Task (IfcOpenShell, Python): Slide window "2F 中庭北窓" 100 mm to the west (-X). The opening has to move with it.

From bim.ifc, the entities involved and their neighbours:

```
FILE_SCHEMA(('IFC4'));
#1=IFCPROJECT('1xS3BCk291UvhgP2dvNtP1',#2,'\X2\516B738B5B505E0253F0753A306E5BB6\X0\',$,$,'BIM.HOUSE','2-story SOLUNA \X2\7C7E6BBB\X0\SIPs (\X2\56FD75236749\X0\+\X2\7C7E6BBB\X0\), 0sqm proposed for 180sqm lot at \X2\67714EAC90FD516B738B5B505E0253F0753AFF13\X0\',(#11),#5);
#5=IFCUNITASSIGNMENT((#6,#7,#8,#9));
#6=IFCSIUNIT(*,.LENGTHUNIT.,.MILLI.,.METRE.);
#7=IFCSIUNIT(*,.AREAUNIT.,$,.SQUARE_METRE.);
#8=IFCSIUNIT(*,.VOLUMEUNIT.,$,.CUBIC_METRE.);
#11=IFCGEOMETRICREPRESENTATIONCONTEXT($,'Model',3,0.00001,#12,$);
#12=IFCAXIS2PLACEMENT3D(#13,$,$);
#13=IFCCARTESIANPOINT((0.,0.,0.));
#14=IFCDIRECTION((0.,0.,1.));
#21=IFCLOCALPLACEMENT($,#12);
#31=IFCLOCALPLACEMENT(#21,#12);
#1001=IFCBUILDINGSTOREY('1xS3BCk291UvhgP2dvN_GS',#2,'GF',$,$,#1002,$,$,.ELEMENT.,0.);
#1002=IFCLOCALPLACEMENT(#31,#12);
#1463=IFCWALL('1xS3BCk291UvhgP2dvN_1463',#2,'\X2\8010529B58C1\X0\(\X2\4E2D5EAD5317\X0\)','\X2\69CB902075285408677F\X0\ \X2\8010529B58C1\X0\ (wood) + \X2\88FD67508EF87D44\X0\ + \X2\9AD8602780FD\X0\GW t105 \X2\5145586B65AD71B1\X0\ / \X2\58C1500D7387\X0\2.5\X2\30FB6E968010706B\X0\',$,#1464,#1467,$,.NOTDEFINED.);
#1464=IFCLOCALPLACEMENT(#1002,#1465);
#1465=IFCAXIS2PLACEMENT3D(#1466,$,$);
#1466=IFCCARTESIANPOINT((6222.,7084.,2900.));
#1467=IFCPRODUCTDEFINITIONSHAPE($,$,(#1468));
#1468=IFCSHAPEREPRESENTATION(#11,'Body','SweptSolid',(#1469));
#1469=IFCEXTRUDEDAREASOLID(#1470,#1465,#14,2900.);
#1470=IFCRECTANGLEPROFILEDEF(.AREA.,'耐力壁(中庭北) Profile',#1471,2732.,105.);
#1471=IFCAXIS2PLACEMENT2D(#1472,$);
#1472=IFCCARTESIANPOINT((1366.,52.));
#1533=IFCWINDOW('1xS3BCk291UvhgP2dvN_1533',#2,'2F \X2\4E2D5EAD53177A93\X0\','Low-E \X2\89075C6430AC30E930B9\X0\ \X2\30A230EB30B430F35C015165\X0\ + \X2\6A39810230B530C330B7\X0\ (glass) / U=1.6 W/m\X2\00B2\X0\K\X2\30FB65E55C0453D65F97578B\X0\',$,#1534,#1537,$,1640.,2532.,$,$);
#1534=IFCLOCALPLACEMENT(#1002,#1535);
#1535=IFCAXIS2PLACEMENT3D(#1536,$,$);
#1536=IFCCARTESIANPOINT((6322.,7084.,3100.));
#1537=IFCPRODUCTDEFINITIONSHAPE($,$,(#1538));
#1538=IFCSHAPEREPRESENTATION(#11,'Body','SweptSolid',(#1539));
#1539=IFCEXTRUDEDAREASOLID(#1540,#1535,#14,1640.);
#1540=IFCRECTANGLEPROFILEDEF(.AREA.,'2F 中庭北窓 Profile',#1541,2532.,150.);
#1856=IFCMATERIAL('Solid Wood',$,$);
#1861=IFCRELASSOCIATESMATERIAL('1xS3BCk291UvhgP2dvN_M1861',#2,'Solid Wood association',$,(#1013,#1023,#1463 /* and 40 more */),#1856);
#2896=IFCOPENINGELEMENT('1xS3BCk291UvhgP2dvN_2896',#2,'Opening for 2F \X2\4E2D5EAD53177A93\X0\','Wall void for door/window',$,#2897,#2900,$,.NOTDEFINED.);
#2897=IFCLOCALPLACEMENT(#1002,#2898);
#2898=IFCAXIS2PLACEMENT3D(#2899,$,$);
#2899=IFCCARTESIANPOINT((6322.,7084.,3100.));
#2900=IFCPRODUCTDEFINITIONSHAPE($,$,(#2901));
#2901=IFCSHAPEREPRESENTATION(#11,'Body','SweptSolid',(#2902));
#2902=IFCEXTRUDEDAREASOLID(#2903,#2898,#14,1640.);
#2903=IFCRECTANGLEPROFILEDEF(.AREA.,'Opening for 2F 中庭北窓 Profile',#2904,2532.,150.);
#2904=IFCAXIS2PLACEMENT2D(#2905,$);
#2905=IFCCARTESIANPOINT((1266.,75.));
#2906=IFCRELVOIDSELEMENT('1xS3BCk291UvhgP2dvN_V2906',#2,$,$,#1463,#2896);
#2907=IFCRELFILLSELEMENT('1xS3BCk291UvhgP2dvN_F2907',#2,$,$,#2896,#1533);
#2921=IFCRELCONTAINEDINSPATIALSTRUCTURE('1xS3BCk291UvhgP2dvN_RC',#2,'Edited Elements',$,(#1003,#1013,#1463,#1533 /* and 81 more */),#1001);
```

```python
import ifcopenshell
import ifcopenshell.api.geometry
import ifcopenshell.util.placement
import ifcopenshell.util.unit

model = ifcopenshell.open("bim.ifc")
unit_scale = ifcopenshell.util.unit.calculate_unit_scale(model)

window = model.by_guid("1xS3BCk291UvhgP2dvN_1533")
opening = window.FillsVoids[0].RelatingOpeningElement
wall = opening.VoidsElements[0].RelatingBuildingElement

wall_matrix = ifcopenshell.util.placement.get_local_placement(wall.ObjectPlacement)
shift = wall_matrix[:3, 0] * -0.1 / unit_scale
before = ifcopenshell.util.placement.get_local_placement(window.ObjectPlacement)[:3, 3].copy()

# The window is not placed relative to its opening, so move both.
for product in (opening, window):
    matrix = ifcopenshell.util.placement.get_local_placement(product.ObjectPlacement)
    matrix[:3, 3] += shift
    ifcopenshell.api.geometry.edit_object_placement(model, product=product, matrix=matrix, is_si=False)

after = ifcopenshell.util.placement.get_local_placement(window.ObjectPlacement)[:3, 3]
print("window moved by", (after - before).round(3) + 0.0)

model.write("bim_updated.ifc")
```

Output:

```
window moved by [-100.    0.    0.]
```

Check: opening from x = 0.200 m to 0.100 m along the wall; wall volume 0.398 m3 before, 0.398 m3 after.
